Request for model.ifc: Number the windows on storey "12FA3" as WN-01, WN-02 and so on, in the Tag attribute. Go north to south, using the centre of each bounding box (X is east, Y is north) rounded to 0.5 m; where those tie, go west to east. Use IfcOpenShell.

First a look at what the model holds.

```python
import ifcopenshell
import ifcopenshell.util.element
import ifcopenshell.util.placement

model = ifcopenshell.open("model.ifc")
print(model.schema)
storey = next(s for s in model.by_type("IfcBuildingStorey") if s.Name == "12FA3")
windows = [e for e in ifcopenshell.util.element.get_decomposition(storey) if e.is_a("IfcWindow")]
for e in sorted(windows, key=lambda e: e.id()):
    origin = ifcopenshell.util.placement.get_local_placement(e.ObjectPlacement)[:3, 3]
    print(e.id(), e.Tag, e.Name, origin.round(2) + 0.0, sep=" | ")
```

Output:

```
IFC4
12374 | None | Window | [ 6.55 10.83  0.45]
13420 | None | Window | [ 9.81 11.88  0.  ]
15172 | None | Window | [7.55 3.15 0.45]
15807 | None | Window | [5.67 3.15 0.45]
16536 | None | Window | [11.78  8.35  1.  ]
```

```python
import ifcopenshell
import ifcopenshell.geom
import ifcopenshell.util.element
import ifcopenshell.util.shape

model = ifcopenshell.open("model.ifc")
settings = ifcopenshell.geom.settings()
settings.set("use-world-coords", True)


def centre(element):
    shape = ifcopenshell.geom.create_shape(settings, element)
    return ifcopenshell.util.shape.get_bbox_centroid(shape.geometry)


storey = next(s for s in model.by_type("IfcBuildingStorey") if s.Name == "12FA3")
windows = [e for e in ifcopenshell.util.element.get_decomposition(storey) if e.is_a("IfcWindow")]

# Insertion points can sit at a corner or the storey origin, so sort by the geometry (in metres).
centres = {e: centre(e) for e in windows}
windows.sort(key=lambda e: (-round(centres[e][1] / 0.5), centres[e][0]))

for i, e in enumerate(windows, start=1):
    number = f"WN-{i:02d}"
    e.Tag = number
    print(e.id(), number)

model.write("model_edited.ifc")
```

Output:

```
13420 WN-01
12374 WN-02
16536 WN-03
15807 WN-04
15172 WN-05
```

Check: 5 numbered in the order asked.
